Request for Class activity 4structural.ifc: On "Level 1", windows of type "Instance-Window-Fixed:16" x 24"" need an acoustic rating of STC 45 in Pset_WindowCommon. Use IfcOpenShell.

First a look at what the model holds.

```python
import ifcopenshell
import ifcopenshell.util.element

model = ifcopenshell.open("Class activity 4structural.ifc")
print(model.schema)
storey = next(s for s in model.by_type("IfcBuildingStorey") if s.Name == "Level 1")
windows = [e for e in ifcopenshell.util.element.get_decomposition(storey) if e.is_a("IfcWindow")]
seen = {}
for e in windows:
    element_type = ifcopenshell.util.element.get_type(e)
    key = (element_type.Name if element_type != e and element_type else None, ifcopenshell.util.element.get_pset(e, "Pset_WindowCommon", "AcousticRating"))
    seen[key] = seen.get(key, 0) + 1
for (name, value), count in sorted(seen.items(), key=str):
    print(count, "x", name, "|", value)
```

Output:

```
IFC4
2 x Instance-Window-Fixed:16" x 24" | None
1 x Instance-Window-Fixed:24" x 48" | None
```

```python
import ifcopenshell
import ifcopenshell.api.pset
import ifcopenshell.util.element

model = ifcopenshell.open("Class activity 4structural.ifc")

storey = next(s for s in model.by_type("IfcBuildingStorey") if s.Name == "Level 1")
windows = [e for e in ifcopenshell.util.element.get_decomposition(storey) if e.is_a("IfcWindow")]

count = 0
for e in windows:
    element_type = ifcopenshell.util.element.get_type(e)
    if element_type in (None, e) or element_type.Name != 'Instance-Window-Fixed:16" x 24"':
        continue
    # add_pset returns the element's existing set when there is one.
    pset = ifcopenshell.api.pset.add_pset(model, product=e, name="Pset_WindowCommon")
    ifcopenshell.api.pset.edit_pset(model, pset=pset, properties={"AcousticRating": "STC 45"})
    count += 1

print(count, "windows updated")

model.write("Class activity 4structural_updated.ifc")
```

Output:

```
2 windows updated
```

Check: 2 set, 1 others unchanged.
